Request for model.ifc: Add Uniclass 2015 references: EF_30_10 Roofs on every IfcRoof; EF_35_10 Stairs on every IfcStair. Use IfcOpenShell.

First a look at what the model holds.

```python
import ifcopenshell

model = ifcopenshell.open("model.ifc")
print(model.schema)
print("classifications:", [c.Name for c in model.by_type("IfcClassification")])
for ifc_class in ("IfcDoor", "IfcRoof", "IfcStair", "IfcWall", "IfcWindow"):
    print(ifc_class, len(model.by_type(ifc_class)))
```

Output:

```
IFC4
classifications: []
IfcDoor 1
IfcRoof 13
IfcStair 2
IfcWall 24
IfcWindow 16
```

```python
import ifcopenshell
import ifcopenshell.api.classification

model = ifcopenshell.open("model.ifc")

system = ifcopenshell.api.classification.add_classification(model, classification="Uniclass 2015")

codes = {
    "IfcRoof": ("EF_30_10", "Roofs"),
    "IfcStair": ("EF_35_10", "Stairs"),
}
for ifc_class, (code, name) in codes.items():
    products = model.by_type(ifc_class)
    ifcopenshell.api.classification.add_reference(
        model, products=products, classification=system, identification=code, name=name
    )
    print(code, len(products))

model.write("model_updated.ifc")
```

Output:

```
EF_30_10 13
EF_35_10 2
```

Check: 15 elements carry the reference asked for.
